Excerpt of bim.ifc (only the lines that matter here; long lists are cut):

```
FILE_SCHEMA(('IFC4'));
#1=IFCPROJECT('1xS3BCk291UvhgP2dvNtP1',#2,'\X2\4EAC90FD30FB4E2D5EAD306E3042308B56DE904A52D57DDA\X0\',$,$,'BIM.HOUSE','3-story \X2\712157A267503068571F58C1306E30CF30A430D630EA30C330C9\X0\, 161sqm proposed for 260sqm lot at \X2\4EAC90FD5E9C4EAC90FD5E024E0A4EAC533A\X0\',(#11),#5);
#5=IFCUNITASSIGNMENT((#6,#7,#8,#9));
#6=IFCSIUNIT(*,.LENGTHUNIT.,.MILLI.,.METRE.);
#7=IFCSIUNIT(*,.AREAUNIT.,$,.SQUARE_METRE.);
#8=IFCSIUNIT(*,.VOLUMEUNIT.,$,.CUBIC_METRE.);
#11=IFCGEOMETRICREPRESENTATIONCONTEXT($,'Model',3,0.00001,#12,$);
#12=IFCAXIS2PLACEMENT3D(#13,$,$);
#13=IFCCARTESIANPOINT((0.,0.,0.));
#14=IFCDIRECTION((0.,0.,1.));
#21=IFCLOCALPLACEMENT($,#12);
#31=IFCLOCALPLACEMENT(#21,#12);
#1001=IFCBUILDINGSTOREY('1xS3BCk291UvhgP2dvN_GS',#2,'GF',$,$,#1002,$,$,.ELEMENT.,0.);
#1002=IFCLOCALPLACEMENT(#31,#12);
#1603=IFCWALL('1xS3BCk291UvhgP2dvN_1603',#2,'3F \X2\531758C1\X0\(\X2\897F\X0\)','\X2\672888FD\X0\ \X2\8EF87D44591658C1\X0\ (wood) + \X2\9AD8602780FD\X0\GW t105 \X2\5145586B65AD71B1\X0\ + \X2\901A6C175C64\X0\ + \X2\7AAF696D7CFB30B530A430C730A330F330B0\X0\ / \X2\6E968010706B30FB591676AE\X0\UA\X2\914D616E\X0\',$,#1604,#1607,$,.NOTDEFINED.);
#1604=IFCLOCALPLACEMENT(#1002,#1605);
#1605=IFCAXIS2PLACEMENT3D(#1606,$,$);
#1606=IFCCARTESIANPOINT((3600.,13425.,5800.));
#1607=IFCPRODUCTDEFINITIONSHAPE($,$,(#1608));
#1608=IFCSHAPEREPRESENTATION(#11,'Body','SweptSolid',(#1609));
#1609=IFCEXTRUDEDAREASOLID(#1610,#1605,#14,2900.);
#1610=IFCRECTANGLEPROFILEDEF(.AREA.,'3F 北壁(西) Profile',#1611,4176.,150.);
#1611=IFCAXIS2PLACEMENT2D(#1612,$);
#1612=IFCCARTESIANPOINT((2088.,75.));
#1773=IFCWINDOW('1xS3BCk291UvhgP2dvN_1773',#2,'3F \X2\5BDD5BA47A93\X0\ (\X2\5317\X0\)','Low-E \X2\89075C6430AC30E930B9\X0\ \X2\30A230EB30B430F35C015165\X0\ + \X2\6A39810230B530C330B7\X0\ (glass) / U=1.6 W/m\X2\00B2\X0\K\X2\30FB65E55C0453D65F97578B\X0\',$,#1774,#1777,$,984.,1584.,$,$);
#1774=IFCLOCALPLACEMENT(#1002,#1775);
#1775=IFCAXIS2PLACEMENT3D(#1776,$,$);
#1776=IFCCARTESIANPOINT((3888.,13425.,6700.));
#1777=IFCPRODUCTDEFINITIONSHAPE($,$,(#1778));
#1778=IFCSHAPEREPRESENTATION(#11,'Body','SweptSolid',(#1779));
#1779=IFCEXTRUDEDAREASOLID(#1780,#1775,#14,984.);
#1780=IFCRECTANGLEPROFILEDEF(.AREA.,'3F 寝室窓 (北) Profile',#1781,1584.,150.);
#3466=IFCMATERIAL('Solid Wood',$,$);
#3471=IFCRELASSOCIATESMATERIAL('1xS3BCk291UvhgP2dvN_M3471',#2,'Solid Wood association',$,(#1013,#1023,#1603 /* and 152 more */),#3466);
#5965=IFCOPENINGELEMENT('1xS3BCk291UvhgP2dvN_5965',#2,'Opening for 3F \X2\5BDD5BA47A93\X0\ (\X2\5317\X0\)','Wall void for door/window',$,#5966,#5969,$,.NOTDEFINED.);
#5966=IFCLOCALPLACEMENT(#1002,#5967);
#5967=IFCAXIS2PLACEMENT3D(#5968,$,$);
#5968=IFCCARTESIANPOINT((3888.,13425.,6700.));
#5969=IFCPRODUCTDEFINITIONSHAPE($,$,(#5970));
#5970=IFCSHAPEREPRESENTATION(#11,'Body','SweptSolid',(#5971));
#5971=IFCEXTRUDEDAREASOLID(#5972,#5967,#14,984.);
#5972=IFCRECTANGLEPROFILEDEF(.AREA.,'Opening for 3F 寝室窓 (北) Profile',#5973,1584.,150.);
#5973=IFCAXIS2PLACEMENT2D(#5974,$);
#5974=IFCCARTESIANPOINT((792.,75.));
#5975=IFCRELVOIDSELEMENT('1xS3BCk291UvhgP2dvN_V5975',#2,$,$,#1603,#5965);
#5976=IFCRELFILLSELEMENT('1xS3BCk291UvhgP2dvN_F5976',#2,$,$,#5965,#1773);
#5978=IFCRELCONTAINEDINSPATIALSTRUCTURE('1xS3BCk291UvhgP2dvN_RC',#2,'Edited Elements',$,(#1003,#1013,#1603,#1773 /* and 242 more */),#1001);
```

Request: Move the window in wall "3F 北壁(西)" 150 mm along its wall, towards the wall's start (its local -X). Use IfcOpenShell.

```python
import ifcopenshell
import ifcopenshell.api.geometry
import ifcopenshell.util.placement

model = ifcopenshell.open("bim.ifc")

window = model.by_guid("1xS3BCk291UvhgP2dvN_1773")
opening = window.FillsVoids[0].RelatingOpeningElement
wall = opening.VoidsElements[0].RelatingBuildingElement

wall_matrix = ifcopenshell.util.placement.get_local_placement(wall.ObjectPlacement)
shift = wall_matrix[:3, 0] * -150.0
before = ifcopenshell.util.placement.get_local_placement(window.ObjectPlacement)[:3, 3].copy()

# The window is not placed relative to its opening, so move both.
for product in (opening, window):
    matrix = ifcopenshell.util.placement.get_local_placement(product.ObjectPlacement)
    matrix[:3, 3] += shift
    ifcopenshell.api.geometry.edit_object_placement(model, product=product, matrix=matrix, is_si=False)

after = ifcopenshell.util.placement.get_local_placement(window.ObjectPlacement)[:3, 3]
print("window moved by", (after - before).round(3) + 0.0)

model.write("bim_updated.ifc")
```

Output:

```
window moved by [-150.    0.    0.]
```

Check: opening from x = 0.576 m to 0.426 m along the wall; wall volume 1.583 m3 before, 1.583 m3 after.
